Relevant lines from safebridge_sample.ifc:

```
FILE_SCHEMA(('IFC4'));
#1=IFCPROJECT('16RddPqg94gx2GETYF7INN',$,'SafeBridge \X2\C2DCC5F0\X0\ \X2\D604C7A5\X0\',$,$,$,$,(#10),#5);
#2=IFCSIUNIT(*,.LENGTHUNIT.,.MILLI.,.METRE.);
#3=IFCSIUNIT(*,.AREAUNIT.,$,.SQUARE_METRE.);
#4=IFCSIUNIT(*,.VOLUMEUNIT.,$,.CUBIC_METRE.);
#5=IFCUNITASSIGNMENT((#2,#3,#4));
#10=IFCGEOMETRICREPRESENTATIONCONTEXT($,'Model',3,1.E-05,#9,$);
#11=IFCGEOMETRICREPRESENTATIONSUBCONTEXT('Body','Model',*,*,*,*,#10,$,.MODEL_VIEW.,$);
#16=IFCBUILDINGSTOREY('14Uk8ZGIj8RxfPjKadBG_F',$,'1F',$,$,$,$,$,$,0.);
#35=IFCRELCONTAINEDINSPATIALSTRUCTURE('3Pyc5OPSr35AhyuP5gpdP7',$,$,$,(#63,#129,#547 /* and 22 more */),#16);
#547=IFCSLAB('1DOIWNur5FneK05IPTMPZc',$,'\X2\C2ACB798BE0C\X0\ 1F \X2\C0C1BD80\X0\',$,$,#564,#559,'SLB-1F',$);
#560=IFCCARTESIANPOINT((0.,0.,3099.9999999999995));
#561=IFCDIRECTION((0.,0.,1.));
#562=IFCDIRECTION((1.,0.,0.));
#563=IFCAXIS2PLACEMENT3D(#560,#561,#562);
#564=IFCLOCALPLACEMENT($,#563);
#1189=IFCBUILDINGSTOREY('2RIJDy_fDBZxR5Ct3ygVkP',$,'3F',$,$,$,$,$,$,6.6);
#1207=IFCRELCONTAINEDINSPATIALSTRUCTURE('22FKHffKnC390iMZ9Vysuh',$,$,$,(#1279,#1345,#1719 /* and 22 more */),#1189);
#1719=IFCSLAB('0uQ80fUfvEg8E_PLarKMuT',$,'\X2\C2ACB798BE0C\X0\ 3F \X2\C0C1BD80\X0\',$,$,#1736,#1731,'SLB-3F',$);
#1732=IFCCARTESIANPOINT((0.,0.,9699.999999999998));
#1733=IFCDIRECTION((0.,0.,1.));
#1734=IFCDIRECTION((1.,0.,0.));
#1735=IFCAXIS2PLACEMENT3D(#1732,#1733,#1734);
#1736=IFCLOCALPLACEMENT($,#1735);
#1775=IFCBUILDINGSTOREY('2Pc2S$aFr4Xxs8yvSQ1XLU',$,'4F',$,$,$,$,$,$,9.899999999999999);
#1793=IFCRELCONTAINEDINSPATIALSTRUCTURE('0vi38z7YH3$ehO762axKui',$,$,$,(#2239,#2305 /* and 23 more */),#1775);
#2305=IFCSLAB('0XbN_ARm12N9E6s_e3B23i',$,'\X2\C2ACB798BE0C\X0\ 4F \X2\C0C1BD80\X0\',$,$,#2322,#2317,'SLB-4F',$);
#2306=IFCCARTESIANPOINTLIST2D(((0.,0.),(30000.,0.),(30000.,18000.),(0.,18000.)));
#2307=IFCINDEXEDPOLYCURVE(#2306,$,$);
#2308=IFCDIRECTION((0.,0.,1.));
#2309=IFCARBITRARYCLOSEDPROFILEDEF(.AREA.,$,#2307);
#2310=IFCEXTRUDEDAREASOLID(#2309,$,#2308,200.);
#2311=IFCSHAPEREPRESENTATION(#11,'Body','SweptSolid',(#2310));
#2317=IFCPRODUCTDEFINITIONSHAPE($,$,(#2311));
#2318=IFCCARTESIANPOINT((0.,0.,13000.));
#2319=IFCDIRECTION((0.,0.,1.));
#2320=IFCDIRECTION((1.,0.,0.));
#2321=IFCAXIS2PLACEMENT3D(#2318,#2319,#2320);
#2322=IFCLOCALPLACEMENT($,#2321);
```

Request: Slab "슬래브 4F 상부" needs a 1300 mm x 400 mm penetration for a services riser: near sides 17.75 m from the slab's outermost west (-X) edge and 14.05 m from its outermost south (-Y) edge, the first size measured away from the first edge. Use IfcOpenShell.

```python
import numpy as np
import ifcopenshell
import ifcopenshell.api.feature
import ifcopenshell.api.geometry
import ifcopenshell.api.root
import ifcopenshell.geom
import ifcopenshell.util.placement
import ifcopenshell.util.representation
import ifcopenshell.util.shape
import ifcopenshell.util.unit

model = ifcopenshell.open("safebridge_sample.ifc")
unit_scale = ifcopenshell.util.unit.calculate_unit_scale(model)
settings = ifcopenshell.geom.settings()


def volume(element):
    """Net volume in cubic metres, openings subtracted."""
    shape = ifcopenshell.geom.create_shape(settings, element)
    return ifcopenshell.util.shape.get_volume(shape.geometry)


slab = model.by_guid("0XbN_ARm12N9E6s_e3B23i")
before = volume(slab)

# Extent in the slab's own axes, in metres. The edges named are its -X and -Y sides.
slab_shape = ifcopenshell.geom.create_shape(settings, slab)
vertices = ifcopenshell.util.shape.get_vertices(slab_shape.geometry)
x_min, y_min, bottom = vertices.min(axis=0)
top = vertices[:, 2].max()

opening = ifcopenshell.api.root.create_entity(model, ifc_class="IfcOpeningElement", name="Services riser opening", predefined_type="OPENING")
context = ifcopenshell.util.representation.get_context(model, "Model", "Body", "MODEL_VIEW")
width, depth = 1.3, 0.4
outline = [(0.0, 0.0), (width, 0.0), (width, depth), (0.0, depth), (0.0, 0.0)]
# Overshoot both faces by 50 mm so the cut is clean.
shape = ifcopenshell.api.geometry.add_slab_representation(
    model, context=context, depth=top - bottom + 0.1, polyline=outline
)
ifcopenshell.api.geometry.assign_representation(model, product=opening, representation=shape)

matrix = ifcopenshell.util.placement.get_local_placement(slab.ObjectPlacement)
matrix[:, 3] = matrix @ np.append(np.array([x_min + 17.75, y_min + 14.05, bottom - 0.05]) / unit_scale, 1.0)
ifcopenshell.api.geometry.edit_object_placement(model, product=opening, matrix=matrix, is_si=False)
ifcopenshell.api.feature.add_feature(model, feature=opening, element=slab)

after = volume(slab)

print(f"slab volume {before:.3f} -> {after:.3f} m3")

model.write("safebridge_sample_v2.ifc")
```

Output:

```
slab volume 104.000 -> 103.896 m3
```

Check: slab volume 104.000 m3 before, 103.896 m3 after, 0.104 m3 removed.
